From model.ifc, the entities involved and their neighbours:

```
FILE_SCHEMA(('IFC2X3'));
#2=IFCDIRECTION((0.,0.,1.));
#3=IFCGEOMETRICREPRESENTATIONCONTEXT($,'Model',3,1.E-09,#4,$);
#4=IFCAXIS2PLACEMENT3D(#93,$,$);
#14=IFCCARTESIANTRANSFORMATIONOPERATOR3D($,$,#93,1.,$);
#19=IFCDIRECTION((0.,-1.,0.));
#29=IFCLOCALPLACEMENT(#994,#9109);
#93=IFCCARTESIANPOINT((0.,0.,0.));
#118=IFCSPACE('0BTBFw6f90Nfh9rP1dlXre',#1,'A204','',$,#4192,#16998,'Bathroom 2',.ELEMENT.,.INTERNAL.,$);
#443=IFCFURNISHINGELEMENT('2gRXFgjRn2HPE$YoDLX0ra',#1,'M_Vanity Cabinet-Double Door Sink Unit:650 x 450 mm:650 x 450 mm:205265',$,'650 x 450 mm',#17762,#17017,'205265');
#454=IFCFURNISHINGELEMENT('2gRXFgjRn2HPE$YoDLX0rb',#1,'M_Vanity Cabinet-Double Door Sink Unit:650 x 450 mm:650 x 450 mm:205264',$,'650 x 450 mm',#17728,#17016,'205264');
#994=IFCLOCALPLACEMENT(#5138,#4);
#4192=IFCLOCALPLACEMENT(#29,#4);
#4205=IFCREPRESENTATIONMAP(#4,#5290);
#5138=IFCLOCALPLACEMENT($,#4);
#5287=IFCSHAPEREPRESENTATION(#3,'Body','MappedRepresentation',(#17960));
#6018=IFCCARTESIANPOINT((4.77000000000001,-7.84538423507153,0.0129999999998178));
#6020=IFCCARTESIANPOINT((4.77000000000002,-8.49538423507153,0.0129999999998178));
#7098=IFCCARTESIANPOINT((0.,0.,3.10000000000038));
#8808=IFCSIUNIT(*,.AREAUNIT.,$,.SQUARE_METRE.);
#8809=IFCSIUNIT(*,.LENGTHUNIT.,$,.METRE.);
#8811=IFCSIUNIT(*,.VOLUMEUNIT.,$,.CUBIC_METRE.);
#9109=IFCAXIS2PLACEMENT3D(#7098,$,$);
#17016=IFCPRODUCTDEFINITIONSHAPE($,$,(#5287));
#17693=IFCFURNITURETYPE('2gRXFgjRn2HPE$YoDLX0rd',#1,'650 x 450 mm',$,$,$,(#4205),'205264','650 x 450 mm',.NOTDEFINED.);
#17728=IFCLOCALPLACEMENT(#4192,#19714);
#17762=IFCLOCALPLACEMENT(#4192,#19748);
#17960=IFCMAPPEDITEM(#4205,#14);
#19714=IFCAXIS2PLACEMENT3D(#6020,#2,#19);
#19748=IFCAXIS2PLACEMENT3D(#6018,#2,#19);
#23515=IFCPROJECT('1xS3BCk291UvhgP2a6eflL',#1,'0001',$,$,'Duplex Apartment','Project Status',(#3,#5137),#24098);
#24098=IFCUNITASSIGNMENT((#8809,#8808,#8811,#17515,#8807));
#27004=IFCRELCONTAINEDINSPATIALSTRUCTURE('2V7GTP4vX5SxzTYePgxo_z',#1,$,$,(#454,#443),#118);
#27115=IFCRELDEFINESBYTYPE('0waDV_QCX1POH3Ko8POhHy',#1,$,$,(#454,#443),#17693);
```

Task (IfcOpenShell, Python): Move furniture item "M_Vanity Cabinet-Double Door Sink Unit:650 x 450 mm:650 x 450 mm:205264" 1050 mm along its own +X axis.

```python
import ifcopenshell
import ifcopenshell.api.geometry
import ifcopenshell.util.placement
import ifcopenshell.util.unit

model = ifcopenshell.open("model.ifc")
unit_scale = ifcopenshell.util.unit.calculate_unit_scale(model)

item = model.by_id(454)
matrix = ifcopenshell.util.placement.get_local_placement(item.ObjectPlacement)
matrix[:3, 3] += matrix[:3, 0] * 1.05 / unit_scale
ifcopenshell.api.geometry.edit_object_placement(model, product=item, matrix=matrix, is_si=False)

print(ifcopenshell.util.placement.get_local_placement(item.ObjectPlacement).round(3) + 0.0)

model.write("model-out.ifc")
```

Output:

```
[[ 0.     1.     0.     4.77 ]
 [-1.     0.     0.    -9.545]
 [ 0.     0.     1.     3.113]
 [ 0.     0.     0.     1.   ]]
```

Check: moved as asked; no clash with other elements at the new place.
